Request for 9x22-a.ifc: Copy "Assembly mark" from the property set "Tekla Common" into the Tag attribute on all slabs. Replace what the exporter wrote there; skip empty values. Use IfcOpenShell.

First a look at what the model holds.

```python
import ifcopenshell
import ifcopenshell.util.element

model = ifcopenshell.open("9x22-a.ifc")
print(model.schema)
slabs = model.by_type("IfcSlab")
print(len(slabs), "slabs")
for e in slabs[:8]:
    source = ifcopenshell.util.element.get_pset(e, "Tekla Common", "Assembly mark")
    target = e.Tag
    print(e.id(), repr(source), repr(target), sep=" | ")
```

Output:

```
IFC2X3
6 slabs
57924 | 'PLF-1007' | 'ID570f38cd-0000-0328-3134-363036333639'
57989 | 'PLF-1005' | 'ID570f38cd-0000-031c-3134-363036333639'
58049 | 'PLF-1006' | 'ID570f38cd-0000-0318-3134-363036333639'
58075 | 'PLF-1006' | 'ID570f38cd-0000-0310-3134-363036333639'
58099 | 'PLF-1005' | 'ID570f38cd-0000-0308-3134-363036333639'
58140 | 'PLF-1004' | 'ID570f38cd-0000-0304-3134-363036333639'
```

```python
import ifcopenshell
import ifcopenshell.util.element

model = ifcopenshell.open("9x22-a.ifc")

count = 0
for e in model.by_type("IfcSlab"):
    value = ifcopenshell.util.element.get_pset(e, "Tekla Common", "Assembly mark")
    current = e.Tag
    if not value or not value.strip() or current == value:
        continue
    e.Tag = value
    count += 1

print(count, "slabs updated")

model.write("9x22-a_edited.ifc")
```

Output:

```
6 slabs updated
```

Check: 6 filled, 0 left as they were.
